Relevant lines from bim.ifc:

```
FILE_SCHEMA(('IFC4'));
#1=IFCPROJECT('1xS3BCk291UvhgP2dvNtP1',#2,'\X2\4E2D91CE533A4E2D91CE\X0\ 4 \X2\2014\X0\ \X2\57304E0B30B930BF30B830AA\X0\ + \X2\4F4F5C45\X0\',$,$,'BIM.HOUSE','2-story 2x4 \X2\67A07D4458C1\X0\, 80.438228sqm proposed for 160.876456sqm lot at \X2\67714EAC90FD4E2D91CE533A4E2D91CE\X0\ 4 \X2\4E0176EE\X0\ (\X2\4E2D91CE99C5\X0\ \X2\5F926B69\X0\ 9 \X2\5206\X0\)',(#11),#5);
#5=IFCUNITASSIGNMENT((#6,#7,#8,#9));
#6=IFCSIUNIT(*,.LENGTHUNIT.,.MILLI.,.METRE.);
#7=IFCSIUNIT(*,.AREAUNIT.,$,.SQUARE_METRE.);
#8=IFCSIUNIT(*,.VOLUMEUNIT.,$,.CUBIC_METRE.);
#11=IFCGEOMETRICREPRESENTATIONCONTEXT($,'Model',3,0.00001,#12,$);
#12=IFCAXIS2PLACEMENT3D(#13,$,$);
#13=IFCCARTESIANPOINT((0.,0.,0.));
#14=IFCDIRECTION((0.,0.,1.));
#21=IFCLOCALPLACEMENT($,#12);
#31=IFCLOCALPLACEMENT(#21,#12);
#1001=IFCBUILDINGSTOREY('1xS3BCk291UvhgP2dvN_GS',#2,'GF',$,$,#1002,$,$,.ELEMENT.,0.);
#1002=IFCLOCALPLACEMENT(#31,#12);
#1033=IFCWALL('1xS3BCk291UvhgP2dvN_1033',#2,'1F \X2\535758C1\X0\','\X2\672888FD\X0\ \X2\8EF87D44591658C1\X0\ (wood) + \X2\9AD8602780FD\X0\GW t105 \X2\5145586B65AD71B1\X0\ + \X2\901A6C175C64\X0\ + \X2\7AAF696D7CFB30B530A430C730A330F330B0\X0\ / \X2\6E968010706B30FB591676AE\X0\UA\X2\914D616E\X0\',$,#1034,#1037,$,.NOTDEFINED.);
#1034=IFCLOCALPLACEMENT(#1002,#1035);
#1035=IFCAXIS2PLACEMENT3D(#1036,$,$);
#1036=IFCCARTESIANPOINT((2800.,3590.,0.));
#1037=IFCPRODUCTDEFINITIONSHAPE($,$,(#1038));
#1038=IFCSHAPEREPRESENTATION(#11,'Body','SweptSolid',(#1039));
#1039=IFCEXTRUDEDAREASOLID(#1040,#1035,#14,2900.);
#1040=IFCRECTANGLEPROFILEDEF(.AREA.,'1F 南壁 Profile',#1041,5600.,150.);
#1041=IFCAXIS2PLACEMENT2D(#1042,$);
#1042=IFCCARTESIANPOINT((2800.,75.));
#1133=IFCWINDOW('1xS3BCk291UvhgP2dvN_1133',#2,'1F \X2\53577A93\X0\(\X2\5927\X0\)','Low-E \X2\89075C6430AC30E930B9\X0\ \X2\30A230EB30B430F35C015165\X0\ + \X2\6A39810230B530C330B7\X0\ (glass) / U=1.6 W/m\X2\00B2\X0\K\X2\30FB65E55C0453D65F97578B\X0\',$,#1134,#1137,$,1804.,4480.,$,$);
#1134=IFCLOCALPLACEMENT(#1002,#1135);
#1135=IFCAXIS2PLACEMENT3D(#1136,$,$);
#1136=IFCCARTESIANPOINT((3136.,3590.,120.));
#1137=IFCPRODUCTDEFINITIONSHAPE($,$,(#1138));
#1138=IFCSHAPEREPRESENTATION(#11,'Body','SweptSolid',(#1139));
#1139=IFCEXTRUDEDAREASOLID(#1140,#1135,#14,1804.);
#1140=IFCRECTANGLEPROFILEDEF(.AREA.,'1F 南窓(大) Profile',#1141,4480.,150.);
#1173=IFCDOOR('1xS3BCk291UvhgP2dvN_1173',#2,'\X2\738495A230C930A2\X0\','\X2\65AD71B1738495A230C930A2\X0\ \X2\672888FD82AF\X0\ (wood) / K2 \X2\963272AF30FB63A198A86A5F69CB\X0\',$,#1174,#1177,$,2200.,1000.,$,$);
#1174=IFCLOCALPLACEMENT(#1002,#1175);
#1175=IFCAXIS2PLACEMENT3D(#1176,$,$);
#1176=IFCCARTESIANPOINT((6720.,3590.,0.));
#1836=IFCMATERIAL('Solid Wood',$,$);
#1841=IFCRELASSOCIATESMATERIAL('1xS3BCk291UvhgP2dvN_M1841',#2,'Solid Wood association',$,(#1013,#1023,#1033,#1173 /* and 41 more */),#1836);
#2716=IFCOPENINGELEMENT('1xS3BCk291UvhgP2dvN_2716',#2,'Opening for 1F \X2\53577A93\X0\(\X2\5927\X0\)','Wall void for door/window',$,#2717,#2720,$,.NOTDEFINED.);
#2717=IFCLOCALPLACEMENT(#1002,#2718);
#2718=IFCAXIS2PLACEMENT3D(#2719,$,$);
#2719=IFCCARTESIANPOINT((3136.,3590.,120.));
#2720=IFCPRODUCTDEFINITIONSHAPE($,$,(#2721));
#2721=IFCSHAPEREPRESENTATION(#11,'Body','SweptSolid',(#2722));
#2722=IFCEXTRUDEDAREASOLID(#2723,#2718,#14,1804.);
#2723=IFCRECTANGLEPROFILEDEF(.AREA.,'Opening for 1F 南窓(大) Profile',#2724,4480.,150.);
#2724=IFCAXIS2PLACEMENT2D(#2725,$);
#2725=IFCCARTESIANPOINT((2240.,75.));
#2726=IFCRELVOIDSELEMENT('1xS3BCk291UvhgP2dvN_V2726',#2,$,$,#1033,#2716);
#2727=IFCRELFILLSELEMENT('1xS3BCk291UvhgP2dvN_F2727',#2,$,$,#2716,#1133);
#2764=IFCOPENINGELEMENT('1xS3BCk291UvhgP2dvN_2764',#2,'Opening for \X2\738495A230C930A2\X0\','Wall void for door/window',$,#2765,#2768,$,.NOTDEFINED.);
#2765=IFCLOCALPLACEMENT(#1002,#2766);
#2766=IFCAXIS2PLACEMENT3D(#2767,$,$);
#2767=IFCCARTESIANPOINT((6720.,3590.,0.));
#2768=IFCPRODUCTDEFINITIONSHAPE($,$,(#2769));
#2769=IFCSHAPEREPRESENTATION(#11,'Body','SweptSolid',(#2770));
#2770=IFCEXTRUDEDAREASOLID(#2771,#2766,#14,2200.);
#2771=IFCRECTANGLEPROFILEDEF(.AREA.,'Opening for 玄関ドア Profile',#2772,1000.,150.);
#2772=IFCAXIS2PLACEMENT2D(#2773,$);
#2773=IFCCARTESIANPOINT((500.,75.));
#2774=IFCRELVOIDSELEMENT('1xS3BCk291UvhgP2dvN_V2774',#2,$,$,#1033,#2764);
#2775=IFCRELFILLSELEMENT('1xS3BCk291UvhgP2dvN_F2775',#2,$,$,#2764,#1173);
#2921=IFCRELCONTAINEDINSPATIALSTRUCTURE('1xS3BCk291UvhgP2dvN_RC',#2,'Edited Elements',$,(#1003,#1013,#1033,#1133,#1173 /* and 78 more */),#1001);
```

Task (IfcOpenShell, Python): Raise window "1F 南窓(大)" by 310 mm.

```python
import numpy as np
import ifcopenshell
import ifcopenshell.api.geometry
import ifcopenshell.util.placement
import ifcopenshell.util.unit

model = ifcopenshell.open("bim.ifc")
unit_scale = ifcopenshell.util.unit.calculate_unit_scale(model)

window = model.by_id(1133)
opening = window.FillsVoids[0].RelatingOpeningElement
dz = 0.31 / unit_scale

shift = np.array([0.0, 0.0, dz])
# The window is not placed relative to its opening, so move both.
for product in (opening, window):
    matrix = ifcopenshell.util.placement.get_local_placement(product.ObjectPlacement)
    matrix[:3, 3] += shift
    ifcopenshell.api.geometry.edit_object_placement(model, product=product, matrix=matrix, is_si=False)

print(f"moved by {dz * unit_scale:+.3f} m")

model.write("bim-out.ifc")
```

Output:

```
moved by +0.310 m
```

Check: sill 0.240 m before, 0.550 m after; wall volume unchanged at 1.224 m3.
